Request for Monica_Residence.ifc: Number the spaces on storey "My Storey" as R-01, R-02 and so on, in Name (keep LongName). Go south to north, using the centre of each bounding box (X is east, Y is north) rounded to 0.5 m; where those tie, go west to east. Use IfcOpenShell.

First a look at what the model holds.

```python
import ifcopenshell
import ifcopenshell.util.element
import ifcopenshell.util.placement

model = ifcopenshell.open("Monica_Residence.ifc")
print(model.schema)
storey = next(s for s in model.by_type("IfcBuildingStorey") if s.Name == "My Storey")
spaces = [e for e in ifcopenshell.util.element.get_decomposition(storey) if e.is_a("IfcSpace")]
for e in sorted(spaces, key=lambda e: e.id()):
    origin = ifcopenshell.util.placement.get_local_placement(e.ObjectPlacement)[:3, 3]
    print(e.id(), e.Name, e.LongName, origin.round(2) + 0.0, sep=" | ")
```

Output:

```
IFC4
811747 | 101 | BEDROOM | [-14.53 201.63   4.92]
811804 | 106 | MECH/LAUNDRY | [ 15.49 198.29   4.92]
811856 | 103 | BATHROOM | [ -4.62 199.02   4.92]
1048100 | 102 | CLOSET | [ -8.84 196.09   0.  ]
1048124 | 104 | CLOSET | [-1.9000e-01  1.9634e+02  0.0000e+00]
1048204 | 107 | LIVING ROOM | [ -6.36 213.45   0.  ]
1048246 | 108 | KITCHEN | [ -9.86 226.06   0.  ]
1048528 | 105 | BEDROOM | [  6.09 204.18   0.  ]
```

```python
import ifcopenshell
import ifcopenshell.geom
import ifcopenshell.util.element
import ifcopenshell.util.shape

model = ifcopenshell.open("Monica_Residence.ifc")
settings = ifcopenshell.geom.settings()
settings.set("use-world-coords", True)


def centre(element):
    shape = ifcopenshell.geom.create_shape(settings, element)
    return ifcopenshell.util.shape.get_bbox_centroid(shape.geometry)


storey = next(s for s in model.by_type("IfcBuildingStorey") if s.Name == "My Storey")
spaces = [e for e in ifcopenshell.util.element.get_decomposition(storey) if e.is_a("IfcSpace")]

# Insertion points can sit at a corner or the storey origin, so sort by the geometry (in metres).
centres = {e: centre(e) for e in spaces}
spaces.sort(key=lambda e: (round(centres[e][1] / 0.5), centres[e][0]))

for i, e in enumerate(spaces, start=1):
    number = f"R-{i:02d}"
    e.Name = number
    print(e.id(), number)

model.write("Monica_Residence_v2.ifc")
```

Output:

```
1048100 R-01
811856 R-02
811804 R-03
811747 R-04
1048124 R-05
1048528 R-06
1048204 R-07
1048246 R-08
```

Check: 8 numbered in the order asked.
